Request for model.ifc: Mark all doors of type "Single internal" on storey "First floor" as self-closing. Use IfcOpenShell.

First a look at what the model holds.

```python
import ifcopenshell
import ifcopenshell.util.element

model = ifcopenshell.open("model.ifc")
print(model.schema)
storey = next(s for s in model.by_type("IfcBuildingStorey") if s.Name == "First floor")
doors = [e for e in ifcopenshell.util.element.get_decomposition(storey) if e.is_a("IfcDoor")]
seen = {}
for e in doors:
    element_type = ifcopenshell.util.element.get_type(e)
    key = (element_type.Name if element_type != e and element_type else None, ifcopenshell.util.element.get_pset(e, "Pset_DoorCommon", "SelfClosing"))
    seen[key] = seen.get(key, 0) + 1
for (name, value), count in sorted(seen.items(), key=str):
    print(count, "x", name, "|", value)
```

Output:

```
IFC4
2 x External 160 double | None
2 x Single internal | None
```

```python
import ifcopenshell
import ifcopenshell.api.pset
import ifcopenshell.util.element

model = ifcopenshell.open("model.ifc")

storey = next(s for s in model.by_type("IfcBuildingStorey") if s.Name == "First floor")
doors = [e for e in ifcopenshell.util.element.get_decomposition(storey) if e.is_a("IfcDoor")]

count = 0
for e in doors:
    element_type = ifcopenshell.util.element.get_type(e)
    if element_type in (None, e) or element_type.Name != "Single internal":
        continue
    # add_pset returns the element's existing set when there is one.
    pset = ifcopenshell.api.pset.add_pset(model, product=e, name="Pset_DoorCommon")
    ifcopenshell.api.pset.edit_pset(model, pset=pset, properties={"SelfClosing": True})
    count += 1

print(count, "doors updated")

model.write("model_rev.ifc")
```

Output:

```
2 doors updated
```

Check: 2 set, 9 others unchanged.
